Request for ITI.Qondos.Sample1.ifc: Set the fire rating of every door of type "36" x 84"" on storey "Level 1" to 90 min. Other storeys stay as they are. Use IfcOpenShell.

First a look at what the model holds.

```python
import ifcopenshell
import ifcopenshell.util.element

model = ifcopenshell.open("ITI.Qondos.Sample1.ifc")
print(model.schema)
storey = next(s for s in model.by_type("IfcBuildingStorey") if s.Name == "Level 1")
doors = [e for e in ifcopenshell.util.element.get_decomposition(storey) if e.is_a("IfcDoor")]
seen = {}
for e in doors:
    element_type = ifcopenshell.util.element.get_type(e)
    key = (element_type.Name if element_type != e and element_type else None, ifcopenshell.util.element.get_pset(e, "Pset_DoorCommon", "FireRating"))
    seen[key] = seen.get(key, 0) + 1
for (name, value), count in sorted(seen.items(), key=str):
    print(count, "x", name, "|", value)
```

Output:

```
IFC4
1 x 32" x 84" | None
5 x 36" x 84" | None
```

```python
import ifcopenshell
import ifcopenshell.api.pset
import ifcopenshell.util.element

model = ifcopenshell.open("ITI.Qondos.Sample1.ifc")

storey = next(s for s in model.by_type("IfcBuildingStorey") if s.Name == "Level 1")
doors = [e for e in ifcopenshell.util.element.get_decomposition(storey) if e.is_a("IfcDoor")]

count = 0
for e in doors:
    element_type = ifcopenshell.util.element.get_type(e)
    if element_type in (None, e) or element_type.Name != '36" x 84"':
        continue
    # add_pset returns the element's existing set when there is one.
    pset = ifcopenshell.api.pset.add_pset(model, product=e, name="Pset_DoorCommon")
    ifcopenshell.api.pset.edit_pset(model, pset=pset, properties={"FireRating": "90 min"})
    count += 1

print(count, "doors updated")

model.write("ITI.Qondos.Sample1_rev.ifc")
```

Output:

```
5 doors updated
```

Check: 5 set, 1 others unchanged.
